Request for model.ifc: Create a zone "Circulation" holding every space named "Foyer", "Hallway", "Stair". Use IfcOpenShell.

First a look at what the model holds.

```python
import ifcopenshell

model = ifcopenshell.open("model.ifc")
print(model.schema)
seen = {}
for space in model.by_type("IfcSpace"):
    seen[space.LongName] = seen.get(space.LongName, 0) + 1
for name, count in sorted(seen.items(), key=str):
    print(count, "x", name)
print("zones:", [z.Name for z in model.by_type("IfcZone")][:20])
```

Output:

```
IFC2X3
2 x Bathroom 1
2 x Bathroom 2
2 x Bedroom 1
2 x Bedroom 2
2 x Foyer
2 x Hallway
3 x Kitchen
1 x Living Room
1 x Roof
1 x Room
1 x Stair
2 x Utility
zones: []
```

```python
import ifcopenshell
import ifcopenshell.api.group
import ifcopenshell.api.root

model = ifcopenshell.open("model.ifc")

names = {"Foyer", "Hallway", "Stair"}
spaces = [s for s in model.by_type("IfcSpace") if s.LongName in names]

zone = ifcopenshell.api.root.create_entity(model, ifc_class="IfcZone", name="Circulation")
ifcopenshell.api.group.assign_group(model, products=spaces, group=zone)
print(len(spaces), "spaces in", zone.Name)

model.write("model_v2.ifc")
```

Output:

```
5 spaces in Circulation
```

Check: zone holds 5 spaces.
